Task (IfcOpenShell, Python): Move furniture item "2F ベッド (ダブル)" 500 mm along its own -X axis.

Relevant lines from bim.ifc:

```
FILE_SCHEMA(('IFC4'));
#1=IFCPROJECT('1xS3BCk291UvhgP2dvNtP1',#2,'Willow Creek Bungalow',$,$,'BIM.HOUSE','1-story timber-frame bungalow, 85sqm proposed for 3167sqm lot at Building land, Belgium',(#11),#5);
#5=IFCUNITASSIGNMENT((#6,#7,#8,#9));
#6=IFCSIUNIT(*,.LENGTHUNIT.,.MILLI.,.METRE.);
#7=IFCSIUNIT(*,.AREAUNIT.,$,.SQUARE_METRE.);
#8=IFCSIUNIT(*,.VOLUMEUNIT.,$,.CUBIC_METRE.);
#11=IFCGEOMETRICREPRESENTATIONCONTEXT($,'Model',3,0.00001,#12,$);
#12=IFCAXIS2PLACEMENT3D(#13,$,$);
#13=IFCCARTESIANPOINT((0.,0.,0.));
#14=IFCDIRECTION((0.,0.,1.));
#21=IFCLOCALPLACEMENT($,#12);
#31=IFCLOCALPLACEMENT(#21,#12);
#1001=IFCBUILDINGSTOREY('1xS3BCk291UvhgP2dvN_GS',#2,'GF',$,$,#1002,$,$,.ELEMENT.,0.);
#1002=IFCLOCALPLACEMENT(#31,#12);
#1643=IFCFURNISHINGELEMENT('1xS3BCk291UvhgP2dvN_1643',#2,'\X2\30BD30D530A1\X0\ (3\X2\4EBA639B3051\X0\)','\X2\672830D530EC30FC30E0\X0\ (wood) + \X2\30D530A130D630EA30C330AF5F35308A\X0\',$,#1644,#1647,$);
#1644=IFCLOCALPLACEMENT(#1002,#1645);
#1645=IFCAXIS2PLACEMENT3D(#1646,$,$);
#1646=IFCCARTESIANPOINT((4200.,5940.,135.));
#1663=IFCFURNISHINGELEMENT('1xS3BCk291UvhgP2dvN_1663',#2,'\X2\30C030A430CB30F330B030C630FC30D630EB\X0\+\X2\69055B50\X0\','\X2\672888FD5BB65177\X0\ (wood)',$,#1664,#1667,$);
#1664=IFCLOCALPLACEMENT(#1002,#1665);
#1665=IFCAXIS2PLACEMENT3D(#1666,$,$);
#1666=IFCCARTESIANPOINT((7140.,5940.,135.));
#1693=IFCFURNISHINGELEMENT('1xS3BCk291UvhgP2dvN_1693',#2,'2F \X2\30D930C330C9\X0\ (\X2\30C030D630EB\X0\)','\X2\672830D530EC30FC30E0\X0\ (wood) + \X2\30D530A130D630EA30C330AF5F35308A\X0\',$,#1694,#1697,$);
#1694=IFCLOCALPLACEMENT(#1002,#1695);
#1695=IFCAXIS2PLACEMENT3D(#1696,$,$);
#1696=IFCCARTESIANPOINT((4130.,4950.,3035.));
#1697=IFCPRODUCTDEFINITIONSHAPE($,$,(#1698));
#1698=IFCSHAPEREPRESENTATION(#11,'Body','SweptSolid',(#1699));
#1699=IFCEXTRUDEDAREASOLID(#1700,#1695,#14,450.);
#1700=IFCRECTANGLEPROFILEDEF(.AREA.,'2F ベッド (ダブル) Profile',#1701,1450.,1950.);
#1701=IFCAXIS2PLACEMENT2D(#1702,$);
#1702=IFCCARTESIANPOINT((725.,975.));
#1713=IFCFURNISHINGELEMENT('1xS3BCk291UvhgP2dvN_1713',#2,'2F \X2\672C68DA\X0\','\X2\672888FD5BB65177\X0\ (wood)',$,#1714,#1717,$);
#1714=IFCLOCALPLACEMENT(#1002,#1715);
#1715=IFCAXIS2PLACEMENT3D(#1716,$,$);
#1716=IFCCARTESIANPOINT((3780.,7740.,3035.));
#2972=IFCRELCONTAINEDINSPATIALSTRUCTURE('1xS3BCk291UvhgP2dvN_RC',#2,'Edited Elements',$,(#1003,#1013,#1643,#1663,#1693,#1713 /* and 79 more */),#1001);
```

```python
import ifcopenshell
import ifcopenshell.api.geometry
import ifcopenshell.util.placement

model = ifcopenshell.open("bim.ifc")

item = model.by_id(1693)
matrix = ifcopenshell.util.placement.get_local_placement(item.ObjectPlacement)
matrix[:3, 3] -= matrix[:3, 0] * 500.0
ifcopenshell.api.geometry.edit_object_placement(model, product=item, matrix=matrix, is_si=False)

print(ifcopenshell.util.placement.get_local_placement(item.ObjectPlacement).round(3) + 0.0)

model.write("bim_v2.ifc")
```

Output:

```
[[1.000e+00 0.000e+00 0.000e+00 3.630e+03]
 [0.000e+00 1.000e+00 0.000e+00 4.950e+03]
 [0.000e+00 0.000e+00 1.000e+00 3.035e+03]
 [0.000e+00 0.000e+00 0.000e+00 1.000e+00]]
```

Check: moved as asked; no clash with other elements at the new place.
